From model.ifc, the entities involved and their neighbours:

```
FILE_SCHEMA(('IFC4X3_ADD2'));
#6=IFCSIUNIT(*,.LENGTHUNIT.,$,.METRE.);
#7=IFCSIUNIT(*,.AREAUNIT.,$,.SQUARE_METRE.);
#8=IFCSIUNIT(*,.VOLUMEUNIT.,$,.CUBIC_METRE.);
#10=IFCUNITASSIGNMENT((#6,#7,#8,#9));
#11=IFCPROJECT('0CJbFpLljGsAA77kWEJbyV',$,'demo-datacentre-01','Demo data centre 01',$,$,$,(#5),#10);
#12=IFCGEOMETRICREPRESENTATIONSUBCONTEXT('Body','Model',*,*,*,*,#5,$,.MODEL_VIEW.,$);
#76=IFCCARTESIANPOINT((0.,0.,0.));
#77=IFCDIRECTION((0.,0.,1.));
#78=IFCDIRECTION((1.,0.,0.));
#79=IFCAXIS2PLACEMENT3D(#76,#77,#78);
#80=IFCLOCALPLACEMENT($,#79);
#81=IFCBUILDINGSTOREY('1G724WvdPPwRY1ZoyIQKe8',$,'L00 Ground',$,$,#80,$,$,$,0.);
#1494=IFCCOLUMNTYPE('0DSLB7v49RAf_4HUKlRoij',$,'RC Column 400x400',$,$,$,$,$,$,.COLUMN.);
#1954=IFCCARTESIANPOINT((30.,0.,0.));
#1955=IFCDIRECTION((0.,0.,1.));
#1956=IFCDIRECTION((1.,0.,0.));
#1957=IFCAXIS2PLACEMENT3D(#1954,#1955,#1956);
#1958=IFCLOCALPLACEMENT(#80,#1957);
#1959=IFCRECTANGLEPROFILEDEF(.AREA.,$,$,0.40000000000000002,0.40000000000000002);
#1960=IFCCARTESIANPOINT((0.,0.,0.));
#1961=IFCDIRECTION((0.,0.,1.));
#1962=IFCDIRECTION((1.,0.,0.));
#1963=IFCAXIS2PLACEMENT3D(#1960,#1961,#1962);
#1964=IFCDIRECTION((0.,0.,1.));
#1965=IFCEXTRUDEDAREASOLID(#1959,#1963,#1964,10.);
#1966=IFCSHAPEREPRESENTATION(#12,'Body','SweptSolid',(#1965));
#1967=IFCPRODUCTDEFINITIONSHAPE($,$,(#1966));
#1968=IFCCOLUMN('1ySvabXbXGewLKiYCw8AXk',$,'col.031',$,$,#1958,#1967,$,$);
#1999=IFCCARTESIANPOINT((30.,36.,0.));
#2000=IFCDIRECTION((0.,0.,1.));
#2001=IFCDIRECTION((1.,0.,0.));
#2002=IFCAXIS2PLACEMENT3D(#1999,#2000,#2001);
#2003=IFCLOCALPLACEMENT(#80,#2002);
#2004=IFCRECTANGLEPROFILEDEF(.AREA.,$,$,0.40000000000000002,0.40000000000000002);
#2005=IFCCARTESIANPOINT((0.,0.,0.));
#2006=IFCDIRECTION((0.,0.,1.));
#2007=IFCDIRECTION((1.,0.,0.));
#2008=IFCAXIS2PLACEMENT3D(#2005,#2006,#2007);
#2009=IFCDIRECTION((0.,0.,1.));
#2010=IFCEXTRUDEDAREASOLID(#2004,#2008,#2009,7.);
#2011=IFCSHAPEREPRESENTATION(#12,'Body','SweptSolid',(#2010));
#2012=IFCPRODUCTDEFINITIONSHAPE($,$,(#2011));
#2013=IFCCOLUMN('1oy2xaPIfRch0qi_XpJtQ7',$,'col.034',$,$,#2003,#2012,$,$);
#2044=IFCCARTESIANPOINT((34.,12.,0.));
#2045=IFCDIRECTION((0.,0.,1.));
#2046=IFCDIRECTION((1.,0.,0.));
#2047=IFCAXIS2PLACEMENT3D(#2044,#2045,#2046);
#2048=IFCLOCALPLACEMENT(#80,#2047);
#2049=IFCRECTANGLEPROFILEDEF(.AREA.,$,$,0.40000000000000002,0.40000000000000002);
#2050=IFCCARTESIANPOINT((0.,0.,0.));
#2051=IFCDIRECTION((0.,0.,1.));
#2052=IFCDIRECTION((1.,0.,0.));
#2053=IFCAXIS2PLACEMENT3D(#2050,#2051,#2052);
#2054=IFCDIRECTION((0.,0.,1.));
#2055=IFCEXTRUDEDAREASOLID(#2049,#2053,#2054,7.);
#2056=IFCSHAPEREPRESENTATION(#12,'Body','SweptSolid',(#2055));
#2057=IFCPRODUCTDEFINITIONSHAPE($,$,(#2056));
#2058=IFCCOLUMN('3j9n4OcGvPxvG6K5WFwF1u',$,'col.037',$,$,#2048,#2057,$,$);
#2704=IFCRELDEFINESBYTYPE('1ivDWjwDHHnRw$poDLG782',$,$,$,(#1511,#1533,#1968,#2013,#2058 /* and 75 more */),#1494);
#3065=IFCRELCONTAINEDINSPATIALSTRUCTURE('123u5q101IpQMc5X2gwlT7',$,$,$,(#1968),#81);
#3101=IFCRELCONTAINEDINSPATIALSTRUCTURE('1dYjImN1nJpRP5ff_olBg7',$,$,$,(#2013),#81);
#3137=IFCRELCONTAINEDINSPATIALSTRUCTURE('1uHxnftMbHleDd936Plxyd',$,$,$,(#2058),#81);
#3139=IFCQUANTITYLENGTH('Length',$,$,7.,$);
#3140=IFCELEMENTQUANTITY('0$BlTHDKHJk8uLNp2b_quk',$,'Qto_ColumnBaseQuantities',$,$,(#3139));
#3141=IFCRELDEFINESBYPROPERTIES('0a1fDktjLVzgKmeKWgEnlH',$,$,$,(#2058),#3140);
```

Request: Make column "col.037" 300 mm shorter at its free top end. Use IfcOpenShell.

```python
import ifcopenshell
import ifcopenshell.api.pset
import ifcopenshell.util.element
import ifcopenshell.util.representation

model = ifcopenshell.open("model.ifc")

member = model.by_guid("3j9n4OcGvPxvG6K5WFwF1u")
change = -0.3

# The extrusion runs towards the end named, so only its depth changes.
body = ifcopenshell.util.representation.get_representation(member, "Model", "Body")
solid = body.Items[0]
old_length = solid.Depth
solid.Depth += change

# Update the stored length and volume.
qto = model.by_id(ifcopenshell.util.element.get_pset(member, "Qto_ColumnBaseQuantities", should_inherit=False)["id"])
ifcopenshell.api.pset.edit_qto(model, qto=qto, properties={"Length": solid.Depth})

print(f"length {old_length:g} -> {solid.Depth:g}")

model.write("model_updated.ifc")
```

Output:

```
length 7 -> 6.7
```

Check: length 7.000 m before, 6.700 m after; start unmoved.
